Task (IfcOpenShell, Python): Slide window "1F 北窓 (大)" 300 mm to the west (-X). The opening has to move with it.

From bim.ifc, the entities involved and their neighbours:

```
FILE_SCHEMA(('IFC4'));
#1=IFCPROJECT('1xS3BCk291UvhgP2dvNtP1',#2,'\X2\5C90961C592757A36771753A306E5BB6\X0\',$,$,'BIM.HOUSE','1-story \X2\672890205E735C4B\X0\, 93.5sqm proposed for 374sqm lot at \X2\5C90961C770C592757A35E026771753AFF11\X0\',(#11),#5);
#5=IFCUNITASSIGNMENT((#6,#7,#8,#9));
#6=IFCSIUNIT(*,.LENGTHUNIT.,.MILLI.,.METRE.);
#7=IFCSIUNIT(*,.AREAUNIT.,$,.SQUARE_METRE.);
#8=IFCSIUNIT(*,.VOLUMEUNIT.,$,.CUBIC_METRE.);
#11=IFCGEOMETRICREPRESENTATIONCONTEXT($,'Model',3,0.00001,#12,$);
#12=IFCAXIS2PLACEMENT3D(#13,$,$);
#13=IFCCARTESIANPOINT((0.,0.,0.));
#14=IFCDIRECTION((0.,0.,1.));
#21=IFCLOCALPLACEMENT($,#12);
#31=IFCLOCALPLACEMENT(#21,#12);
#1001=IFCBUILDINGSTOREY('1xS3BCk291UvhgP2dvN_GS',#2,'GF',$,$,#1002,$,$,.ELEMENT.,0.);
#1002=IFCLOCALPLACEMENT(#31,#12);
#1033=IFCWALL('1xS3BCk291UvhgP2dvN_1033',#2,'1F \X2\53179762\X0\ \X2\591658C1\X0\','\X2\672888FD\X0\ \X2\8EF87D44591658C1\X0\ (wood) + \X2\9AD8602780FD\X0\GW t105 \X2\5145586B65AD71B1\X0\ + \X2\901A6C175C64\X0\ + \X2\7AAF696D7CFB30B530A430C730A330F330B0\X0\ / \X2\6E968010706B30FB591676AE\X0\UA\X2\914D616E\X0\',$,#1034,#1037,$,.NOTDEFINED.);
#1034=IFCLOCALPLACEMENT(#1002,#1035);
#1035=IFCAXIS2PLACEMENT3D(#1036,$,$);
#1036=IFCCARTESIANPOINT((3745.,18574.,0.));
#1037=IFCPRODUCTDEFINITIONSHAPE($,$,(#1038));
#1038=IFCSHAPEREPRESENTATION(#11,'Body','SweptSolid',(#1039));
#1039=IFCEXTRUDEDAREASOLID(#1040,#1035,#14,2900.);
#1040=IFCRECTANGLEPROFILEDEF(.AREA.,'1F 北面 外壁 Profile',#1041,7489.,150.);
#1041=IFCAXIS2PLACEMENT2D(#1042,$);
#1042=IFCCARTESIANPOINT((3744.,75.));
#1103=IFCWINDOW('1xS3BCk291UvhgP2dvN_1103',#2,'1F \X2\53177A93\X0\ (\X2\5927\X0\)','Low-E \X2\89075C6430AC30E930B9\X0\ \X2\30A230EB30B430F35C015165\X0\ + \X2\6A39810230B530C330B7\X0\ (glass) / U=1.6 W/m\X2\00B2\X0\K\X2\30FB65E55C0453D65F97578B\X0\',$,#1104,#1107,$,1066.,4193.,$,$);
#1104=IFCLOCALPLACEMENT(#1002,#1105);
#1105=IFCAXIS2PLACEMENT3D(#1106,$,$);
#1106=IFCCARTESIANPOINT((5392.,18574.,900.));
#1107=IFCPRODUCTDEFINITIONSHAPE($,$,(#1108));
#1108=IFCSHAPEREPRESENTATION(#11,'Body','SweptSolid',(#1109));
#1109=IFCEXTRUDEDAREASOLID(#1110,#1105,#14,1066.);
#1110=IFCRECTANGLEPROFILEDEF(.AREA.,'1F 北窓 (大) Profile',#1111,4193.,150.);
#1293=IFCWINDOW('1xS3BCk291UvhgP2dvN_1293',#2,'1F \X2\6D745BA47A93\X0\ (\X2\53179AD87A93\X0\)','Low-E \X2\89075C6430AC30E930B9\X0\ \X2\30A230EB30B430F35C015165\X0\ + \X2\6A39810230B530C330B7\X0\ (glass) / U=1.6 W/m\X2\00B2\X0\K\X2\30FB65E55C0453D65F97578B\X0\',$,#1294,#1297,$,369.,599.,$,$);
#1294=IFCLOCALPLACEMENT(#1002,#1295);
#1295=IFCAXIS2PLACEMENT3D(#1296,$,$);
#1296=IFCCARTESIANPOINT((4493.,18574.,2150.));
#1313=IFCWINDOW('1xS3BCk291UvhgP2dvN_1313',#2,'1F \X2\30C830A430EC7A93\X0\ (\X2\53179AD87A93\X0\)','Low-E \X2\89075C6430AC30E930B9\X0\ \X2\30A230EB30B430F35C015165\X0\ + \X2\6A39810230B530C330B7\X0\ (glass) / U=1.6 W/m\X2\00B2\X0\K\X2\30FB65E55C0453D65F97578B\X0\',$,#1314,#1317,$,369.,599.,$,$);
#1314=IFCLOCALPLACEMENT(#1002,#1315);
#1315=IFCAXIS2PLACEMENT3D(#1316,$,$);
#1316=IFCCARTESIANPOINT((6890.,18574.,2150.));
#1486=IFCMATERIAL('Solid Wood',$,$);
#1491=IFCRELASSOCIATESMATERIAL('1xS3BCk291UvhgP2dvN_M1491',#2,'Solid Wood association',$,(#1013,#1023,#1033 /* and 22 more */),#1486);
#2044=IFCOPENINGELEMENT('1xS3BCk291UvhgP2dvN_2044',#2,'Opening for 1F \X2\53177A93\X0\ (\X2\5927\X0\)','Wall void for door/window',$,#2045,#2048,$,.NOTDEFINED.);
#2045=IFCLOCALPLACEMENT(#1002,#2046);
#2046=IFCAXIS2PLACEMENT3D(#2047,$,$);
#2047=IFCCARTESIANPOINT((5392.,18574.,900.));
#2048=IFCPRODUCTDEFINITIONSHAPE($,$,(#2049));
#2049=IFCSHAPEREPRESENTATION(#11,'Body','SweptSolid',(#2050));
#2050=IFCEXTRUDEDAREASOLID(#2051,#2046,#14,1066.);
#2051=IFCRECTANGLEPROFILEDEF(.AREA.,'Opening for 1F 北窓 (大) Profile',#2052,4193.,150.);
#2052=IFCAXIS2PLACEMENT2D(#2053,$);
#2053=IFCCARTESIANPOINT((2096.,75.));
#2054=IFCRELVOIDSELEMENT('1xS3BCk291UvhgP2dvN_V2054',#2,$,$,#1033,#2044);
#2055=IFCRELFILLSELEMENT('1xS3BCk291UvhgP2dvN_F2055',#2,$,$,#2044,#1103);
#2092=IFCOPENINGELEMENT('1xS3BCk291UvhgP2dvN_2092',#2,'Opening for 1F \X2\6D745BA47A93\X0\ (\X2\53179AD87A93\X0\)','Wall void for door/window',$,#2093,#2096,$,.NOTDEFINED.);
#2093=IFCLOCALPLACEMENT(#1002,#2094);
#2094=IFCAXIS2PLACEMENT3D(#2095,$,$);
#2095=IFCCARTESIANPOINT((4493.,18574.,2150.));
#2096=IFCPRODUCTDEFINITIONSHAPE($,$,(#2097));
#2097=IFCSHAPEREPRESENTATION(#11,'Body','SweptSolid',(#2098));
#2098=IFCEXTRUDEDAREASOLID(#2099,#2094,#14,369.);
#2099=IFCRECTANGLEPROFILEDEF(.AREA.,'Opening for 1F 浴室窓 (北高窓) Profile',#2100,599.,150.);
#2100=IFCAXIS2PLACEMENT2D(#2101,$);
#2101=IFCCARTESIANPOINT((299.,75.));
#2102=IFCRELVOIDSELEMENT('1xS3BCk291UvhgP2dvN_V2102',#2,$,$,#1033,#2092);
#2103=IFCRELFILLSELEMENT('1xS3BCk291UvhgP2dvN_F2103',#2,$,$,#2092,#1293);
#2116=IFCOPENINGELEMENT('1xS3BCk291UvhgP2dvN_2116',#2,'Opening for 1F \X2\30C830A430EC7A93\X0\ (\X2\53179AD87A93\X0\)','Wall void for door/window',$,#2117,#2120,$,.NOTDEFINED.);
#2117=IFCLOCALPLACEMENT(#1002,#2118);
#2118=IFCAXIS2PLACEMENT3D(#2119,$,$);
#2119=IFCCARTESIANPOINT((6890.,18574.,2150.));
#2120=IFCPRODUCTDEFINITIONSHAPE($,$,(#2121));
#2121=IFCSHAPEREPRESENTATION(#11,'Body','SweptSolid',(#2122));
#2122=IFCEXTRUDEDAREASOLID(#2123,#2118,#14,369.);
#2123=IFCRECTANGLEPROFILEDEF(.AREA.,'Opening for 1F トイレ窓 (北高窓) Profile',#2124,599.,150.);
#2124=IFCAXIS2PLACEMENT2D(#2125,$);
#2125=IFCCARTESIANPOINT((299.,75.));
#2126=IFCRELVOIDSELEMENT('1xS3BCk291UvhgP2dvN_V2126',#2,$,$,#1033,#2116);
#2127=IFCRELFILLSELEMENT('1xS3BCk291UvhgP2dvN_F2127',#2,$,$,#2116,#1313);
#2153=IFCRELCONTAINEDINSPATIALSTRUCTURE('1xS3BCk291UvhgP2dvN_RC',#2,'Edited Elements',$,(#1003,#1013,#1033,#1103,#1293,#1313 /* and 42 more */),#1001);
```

```python
import ifcopenshell
import ifcopenshell.api.geometry
import ifcopenshell.util.placement
import ifcopenshell.util.unit

model = ifcopenshell.open("bim.ifc")
unit_scale = ifcopenshell.util.unit.calculate_unit_scale(model)

window = model.by_guid("1xS3BCk291UvhgP2dvN_1103")
opening = window.FillsVoids[0].RelatingOpeningElement
wall = opening.VoidsElements[0].RelatingBuildingElement

wall_matrix = ifcopenshell.util.placement.get_local_placement(wall.ObjectPlacement)
shift = wall_matrix[:3, 0] * -0.3 / unit_scale
before = ifcopenshell.util.placement.get_local_placement(window.ObjectPlacement)[:3, 3].copy()

# The window is not placed relative to its opening, so move both.
for product in (opening, window):
    matrix = ifcopenshell.util.placement.get_local_placement(product.ObjectPlacement)
    matrix[:3, 3] += shift
    ifcopenshell.api.geometry.edit_object_placement(model, product=product, matrix=matrix, is_si=False)

after = ifcopenshell.util.placement.get_local_placement(window.ObjectPlacement)[:3, 3]
print("window moved by", (after - before).round(3) + 0.0)

model.write("bim-out.ifc")
```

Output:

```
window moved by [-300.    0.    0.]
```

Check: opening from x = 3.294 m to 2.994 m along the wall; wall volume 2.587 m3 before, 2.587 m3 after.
